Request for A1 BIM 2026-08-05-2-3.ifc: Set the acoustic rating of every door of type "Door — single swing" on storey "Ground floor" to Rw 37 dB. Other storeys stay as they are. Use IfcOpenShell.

First a look at what the model holds.

```python
import ifcopenshell
import ifcopenshell.util.element

model = ifcopenshell.open("A1 BIM 2026-08-05-2-3.ifc")
print(model.schema)
storey = next(s for s in model.by_type("IfcBuildingStorey") if s.Name == "Ground floor")
doors = [e for e in ifcopenshell.util.element.get_decomposition(storey) if e.is_a("IfcDoor")]
seen = {}
for e in doors:
    element_type = ifcopenshell.util.element.get_type(e)
    key = (element_type.Name if element_type != e and element_type else None, ifcopenshell.util.element.get_pset(e, "Pset_DoorCommon", "AcousticRating"))
    seen[key] = seen.get(key, 0) + 1
for (name, value), count in sorted(seen.items(), key=str):
    print(count, "x", name, "|", value)
```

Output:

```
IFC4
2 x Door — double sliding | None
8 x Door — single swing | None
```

```python
import ifcopenshell
import ifcopenshell.api.pset
import ifcopenshell.util.element

model = ifcopenshell.open("A1 BIM 2026-08-05-2-3.ifc")

storey = next(s for s in model.by_type("IfcBuildingStorey") if s.Name == "Ground floor")
doors = [e for e in ifcopenshell.util.element.get_decomposition(storey) if e.is_a("IfcDoor")]

count = 0
for e in doors:
    element_type = ifcopenshell.util.element.get_type(e)
    if element_type in (None, e) or element_type.Name != "Door — single swing":
        continue
    # add_pset returns the element's existing set when there is one.
    pset = ifcopenshell.api.pset.add_pset(model, product=e, name="Pset_DoorCommon")
    ifcopenshell.api.pset.edit_pset(model, pset=pset, properties={"AcousticRating": "Rw 37 dB"})
    count += 1

print(count, "doors updated")

model.write("A1 BIM 2026-08-05-2-3_rev.ifc")
```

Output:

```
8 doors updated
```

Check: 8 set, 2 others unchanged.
